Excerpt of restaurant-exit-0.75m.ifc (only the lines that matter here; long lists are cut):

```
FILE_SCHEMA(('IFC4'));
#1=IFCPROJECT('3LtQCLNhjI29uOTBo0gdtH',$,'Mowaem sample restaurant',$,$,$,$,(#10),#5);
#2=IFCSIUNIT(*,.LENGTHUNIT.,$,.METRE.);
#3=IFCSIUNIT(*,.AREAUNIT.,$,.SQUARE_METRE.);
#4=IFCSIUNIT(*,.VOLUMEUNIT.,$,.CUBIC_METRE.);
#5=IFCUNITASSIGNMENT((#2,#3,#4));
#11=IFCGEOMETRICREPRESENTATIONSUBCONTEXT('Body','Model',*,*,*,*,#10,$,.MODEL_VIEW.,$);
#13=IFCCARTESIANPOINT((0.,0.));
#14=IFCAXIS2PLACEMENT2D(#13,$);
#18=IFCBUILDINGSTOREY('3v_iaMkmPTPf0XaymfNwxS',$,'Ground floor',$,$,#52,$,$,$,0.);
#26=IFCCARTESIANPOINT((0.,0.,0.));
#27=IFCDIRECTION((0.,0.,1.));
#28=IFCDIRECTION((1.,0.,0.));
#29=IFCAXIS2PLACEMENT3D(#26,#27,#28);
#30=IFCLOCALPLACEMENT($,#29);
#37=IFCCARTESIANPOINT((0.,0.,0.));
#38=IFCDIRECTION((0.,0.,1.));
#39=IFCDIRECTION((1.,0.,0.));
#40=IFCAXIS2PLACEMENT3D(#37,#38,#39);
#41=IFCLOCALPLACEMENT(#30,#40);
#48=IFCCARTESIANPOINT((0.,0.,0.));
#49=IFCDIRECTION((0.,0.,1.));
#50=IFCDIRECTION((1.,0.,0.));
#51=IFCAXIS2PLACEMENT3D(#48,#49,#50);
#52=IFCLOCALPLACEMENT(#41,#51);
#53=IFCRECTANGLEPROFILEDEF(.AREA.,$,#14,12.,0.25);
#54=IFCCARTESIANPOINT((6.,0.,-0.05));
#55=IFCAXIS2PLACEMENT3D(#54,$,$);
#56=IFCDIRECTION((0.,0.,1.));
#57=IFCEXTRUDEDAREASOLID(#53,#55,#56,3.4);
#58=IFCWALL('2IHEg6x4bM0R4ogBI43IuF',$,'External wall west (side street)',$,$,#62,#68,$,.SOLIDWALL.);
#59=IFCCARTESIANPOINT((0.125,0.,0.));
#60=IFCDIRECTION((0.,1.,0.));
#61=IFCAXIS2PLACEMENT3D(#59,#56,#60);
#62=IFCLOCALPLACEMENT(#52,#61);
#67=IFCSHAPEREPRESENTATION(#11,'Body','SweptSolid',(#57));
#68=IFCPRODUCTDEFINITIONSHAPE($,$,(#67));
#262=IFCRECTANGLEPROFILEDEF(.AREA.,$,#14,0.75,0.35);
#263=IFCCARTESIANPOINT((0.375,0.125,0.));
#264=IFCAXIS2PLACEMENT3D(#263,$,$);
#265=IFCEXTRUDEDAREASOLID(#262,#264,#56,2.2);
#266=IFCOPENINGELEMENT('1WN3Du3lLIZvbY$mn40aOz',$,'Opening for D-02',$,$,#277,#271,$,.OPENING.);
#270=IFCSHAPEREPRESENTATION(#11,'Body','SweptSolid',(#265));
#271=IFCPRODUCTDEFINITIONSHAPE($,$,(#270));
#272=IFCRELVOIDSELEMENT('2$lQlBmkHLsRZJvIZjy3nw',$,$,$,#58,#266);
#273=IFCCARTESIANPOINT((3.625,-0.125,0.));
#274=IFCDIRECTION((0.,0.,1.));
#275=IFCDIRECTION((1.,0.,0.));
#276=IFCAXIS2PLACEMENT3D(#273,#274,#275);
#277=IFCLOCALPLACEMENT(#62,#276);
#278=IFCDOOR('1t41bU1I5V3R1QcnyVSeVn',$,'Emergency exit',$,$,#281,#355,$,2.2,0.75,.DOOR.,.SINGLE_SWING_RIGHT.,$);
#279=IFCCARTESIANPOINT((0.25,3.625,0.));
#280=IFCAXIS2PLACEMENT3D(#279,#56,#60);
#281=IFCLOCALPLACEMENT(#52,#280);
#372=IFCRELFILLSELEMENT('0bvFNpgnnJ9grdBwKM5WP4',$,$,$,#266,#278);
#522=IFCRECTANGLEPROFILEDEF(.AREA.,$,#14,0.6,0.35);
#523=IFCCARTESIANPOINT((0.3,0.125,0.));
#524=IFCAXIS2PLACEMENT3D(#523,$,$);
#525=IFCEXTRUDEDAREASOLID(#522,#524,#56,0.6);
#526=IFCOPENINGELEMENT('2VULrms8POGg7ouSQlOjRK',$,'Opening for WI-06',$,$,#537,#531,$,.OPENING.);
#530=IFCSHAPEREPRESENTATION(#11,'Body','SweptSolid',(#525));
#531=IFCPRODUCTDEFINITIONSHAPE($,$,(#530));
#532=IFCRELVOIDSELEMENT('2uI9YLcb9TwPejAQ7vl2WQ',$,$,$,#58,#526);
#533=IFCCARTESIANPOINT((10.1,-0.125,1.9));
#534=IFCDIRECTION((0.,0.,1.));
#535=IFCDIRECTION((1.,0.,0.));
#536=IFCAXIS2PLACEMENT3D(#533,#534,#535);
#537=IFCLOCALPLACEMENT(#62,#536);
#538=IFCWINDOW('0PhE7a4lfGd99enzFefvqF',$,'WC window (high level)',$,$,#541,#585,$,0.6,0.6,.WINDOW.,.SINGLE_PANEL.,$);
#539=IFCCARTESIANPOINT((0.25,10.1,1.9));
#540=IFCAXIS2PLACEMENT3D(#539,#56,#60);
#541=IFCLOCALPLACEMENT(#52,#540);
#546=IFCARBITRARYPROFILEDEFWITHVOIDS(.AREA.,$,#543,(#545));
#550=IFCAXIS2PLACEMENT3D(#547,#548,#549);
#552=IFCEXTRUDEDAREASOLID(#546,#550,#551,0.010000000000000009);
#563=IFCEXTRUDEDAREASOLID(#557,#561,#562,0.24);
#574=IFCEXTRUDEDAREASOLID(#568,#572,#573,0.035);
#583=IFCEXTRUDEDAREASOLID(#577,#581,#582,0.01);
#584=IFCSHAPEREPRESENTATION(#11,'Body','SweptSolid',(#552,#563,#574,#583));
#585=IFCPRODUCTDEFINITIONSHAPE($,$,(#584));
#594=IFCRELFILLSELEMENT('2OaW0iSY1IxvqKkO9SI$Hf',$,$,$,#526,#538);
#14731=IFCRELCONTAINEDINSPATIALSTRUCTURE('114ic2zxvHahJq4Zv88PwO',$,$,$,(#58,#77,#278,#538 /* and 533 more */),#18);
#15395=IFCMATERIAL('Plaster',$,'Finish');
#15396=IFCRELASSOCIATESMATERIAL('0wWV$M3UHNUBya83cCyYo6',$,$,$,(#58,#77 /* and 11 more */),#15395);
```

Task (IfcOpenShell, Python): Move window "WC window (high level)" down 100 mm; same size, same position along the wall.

```python
import numpy as np
import ifcopenshell
import ifcopenshell.api.geometry
import ifcopenshell.util.placement
import ifcopenshell.util.unit

model = ifcopenshell.open("restaurant-exit-0.75m.ifc")
unit_scale = ifcopenshell.util.unit.calculate_unit_scale(model)

window = model.by_id(538)
opening = window.FillsVoids[0].RelatingOpeningElement
dz = -0.1 / unit_scale

shift = np.array([0.0, 0.0, dz])
# The window is not placed relative to its opening, so move both.
for product in (opening, window):
    matrix = ifcopenshell.util.placement.get_local_placement(product.ObjectPlacement)
    matrix[:3, 3] += shift
    ifcopenshell.api.geometry.edit_object_placement(model, product=product, matrix=matrix, is_si=False)

print(f"moved by {dz * unit_scale:+.3f} m")

model.write("restaurant-exit-0.75m_edited.ifc")
```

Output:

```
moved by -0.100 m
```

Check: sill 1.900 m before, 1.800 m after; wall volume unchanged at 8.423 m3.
